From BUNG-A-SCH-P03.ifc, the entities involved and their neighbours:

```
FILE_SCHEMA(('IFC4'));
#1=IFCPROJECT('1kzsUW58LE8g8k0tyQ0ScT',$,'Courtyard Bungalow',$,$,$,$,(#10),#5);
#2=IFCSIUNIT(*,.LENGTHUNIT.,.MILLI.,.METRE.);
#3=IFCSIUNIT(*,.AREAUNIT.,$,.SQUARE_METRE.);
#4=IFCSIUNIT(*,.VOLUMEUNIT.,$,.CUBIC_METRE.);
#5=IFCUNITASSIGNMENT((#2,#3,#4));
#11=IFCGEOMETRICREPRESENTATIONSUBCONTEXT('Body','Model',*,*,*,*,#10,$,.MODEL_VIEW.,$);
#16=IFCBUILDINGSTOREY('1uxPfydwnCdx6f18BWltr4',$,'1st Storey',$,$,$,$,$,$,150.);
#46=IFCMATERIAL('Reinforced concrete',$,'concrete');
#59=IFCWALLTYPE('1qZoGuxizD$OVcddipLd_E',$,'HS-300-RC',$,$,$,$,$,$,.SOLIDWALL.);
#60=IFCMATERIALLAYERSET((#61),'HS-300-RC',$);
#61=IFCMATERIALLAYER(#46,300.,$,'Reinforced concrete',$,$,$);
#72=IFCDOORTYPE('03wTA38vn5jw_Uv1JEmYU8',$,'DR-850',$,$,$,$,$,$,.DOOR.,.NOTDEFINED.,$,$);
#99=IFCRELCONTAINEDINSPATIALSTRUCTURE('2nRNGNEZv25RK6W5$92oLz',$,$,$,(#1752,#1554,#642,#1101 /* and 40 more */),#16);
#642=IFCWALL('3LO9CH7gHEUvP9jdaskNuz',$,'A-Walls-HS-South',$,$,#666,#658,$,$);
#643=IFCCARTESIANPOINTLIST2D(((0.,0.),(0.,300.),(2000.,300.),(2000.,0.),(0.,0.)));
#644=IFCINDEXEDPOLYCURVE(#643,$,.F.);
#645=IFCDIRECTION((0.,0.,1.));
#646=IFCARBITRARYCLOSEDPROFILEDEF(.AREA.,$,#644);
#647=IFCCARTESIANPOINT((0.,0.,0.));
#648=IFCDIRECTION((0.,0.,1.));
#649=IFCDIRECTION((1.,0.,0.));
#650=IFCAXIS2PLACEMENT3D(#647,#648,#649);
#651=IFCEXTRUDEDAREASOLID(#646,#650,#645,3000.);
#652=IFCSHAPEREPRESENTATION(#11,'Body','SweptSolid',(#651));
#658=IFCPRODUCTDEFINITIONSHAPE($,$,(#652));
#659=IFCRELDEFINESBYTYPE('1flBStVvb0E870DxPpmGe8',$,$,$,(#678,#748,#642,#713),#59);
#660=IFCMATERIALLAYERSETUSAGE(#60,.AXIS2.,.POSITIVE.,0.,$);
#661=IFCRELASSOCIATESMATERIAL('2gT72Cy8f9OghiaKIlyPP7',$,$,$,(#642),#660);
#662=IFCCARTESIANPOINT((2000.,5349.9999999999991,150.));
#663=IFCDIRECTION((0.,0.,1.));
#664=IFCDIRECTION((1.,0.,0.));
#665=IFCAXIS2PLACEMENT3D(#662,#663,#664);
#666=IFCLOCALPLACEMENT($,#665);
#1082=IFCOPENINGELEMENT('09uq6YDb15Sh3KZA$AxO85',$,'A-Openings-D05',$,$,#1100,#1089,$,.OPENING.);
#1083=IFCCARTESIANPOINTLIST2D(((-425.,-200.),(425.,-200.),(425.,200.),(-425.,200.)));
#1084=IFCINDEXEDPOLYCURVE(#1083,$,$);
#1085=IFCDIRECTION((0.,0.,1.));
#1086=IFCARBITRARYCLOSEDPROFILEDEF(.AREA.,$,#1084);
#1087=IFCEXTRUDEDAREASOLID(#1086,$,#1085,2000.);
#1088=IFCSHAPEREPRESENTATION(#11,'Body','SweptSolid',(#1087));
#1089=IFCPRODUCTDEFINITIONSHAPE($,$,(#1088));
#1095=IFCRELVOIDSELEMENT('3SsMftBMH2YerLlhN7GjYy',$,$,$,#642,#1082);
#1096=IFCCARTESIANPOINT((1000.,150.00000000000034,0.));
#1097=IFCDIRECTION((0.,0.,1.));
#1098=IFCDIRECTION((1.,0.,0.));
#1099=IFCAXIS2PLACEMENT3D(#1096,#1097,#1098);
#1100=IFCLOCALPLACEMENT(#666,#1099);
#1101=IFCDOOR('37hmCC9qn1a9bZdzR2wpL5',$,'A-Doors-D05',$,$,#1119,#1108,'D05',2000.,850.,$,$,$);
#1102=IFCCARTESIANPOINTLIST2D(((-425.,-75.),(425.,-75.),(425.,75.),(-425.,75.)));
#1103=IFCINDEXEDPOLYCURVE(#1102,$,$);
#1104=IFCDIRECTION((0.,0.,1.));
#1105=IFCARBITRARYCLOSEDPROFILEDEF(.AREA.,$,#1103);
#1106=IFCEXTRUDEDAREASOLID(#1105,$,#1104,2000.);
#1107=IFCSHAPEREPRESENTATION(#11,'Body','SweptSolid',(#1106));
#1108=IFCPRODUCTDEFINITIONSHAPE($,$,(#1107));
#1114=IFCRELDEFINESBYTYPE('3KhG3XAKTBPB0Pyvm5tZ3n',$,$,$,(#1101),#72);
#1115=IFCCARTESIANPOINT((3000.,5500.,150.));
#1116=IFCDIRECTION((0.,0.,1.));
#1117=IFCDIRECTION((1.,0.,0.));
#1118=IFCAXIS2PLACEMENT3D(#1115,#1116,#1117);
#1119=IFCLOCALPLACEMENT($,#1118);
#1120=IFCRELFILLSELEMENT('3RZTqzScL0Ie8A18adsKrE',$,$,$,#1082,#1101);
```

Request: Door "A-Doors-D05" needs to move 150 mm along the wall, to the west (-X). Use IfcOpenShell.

```python
import ifcopenshell
import ifcopenshell.api.geometry
import ifcopenshell.util.placement
import ifcopenshell.util.unit

model = ifcopenshell.open("BUNG-A-SCH-P03.ifc")
unit_scale = ifcopenshell.util.unit.calculate_unit_scale(model)

door = model.by_guid("37hmCC9qn1a9bZdzR2wpL5")
opening = door.FillsVoids[0].RelatingOpeningElement
wall = opening.VoidsElements[0].RelatingBuildingElement

wall_matrix = ifcopenshell.util.placement.get_local_placement(wall.ObjectPlacement)
shift = wall_matrix[:3, 0] * -0.15 / unit_scale
before = ifcopenshell.util.placement.get_local_placement(door.ObjectPlacement)[:3, 3].copy()

# The door is not placed relative to its opening, so move both.
for product in (opening, door):
    matrix = ifcopenshell.util.placement.get_local_placement(product.ObjectPlacement)
    matrix[:3, 3] += shift
    ifcopenshell.api.geometry.edit_object_placement(model, product=product, matrix=matrix, is_si=False)

after = ifcopenshell.util.placement.get_local_placement(door.ObjectPlacement)[:3, 3]
print("door moved by", (after - before).round(3) + 0.0)

model.write("BUNG-A-SCH-P03_v2.ifc")
```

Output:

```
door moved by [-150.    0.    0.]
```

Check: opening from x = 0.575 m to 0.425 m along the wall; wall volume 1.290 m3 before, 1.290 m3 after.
